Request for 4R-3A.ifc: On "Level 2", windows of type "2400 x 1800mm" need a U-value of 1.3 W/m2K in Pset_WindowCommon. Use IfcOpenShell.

First a look at what the model holds.

```python
import ifcopenshell
import ifcopenshell.util.element

model = ifcopenshell.open("4R-3A.ifc")
print(model.schema)
storey = next(s for s in model.by_type("IfcBuildingStorey") if s.Name == "Level 2")
windows = [e for e in ifcopenshell.util.element.get_decomposition(storey) if e.is_a("IfcWindow")]
seen = {}
for e in windows:
    element_type = ifcopenshell.util.element.get_type(e)
    key = (element_type.Name if element_type != e and element_type else None, ifcopenshell.util.element.get_pset(e, "Pset_WindowCommon", "ThermalTransmittance"))
    seen[key] = seen.get(key, 0) + 1
for (name, value), count in sorted(seen.items(), key=str):
    print(count, "x", name, "|", value)
```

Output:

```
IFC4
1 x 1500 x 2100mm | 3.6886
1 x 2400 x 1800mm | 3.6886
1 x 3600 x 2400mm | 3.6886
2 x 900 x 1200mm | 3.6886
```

```python
import ifcopenshell
import ifcopenshell.api.pset
import ifcopenshell.util.element

model = ifcopenshell.open("4R-3A.ifc")

storey = next(s for s in model.by_type("IfcBuildingStorey") if s.Name == "Level 2")
windows = [e for e in ifcopenshell.util.element.get_decomposition(storey) if e.is_a("IfcWindow")]

count = 0
for e in windows:
    element_type = ifcopenshell.util.element.get_type(e)
    if element_type in (None, e) or element_type.Name != "2400 x 1800mm":
        continue
    # add_pset returns the element's existing set when there is one.
    pset = ifcopenshell.api.pset.add_pset(model, product=e, name="Pset_WindowCommon")
    ifcopenshell.api.pset.edit_pset(model, pset=pset, properties={"ThermalTransmittance": 1.3})
    count += 1

print(count, "windows updated")

model.write("4R-3A_updated.ifc")
```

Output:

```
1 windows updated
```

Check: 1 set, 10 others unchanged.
